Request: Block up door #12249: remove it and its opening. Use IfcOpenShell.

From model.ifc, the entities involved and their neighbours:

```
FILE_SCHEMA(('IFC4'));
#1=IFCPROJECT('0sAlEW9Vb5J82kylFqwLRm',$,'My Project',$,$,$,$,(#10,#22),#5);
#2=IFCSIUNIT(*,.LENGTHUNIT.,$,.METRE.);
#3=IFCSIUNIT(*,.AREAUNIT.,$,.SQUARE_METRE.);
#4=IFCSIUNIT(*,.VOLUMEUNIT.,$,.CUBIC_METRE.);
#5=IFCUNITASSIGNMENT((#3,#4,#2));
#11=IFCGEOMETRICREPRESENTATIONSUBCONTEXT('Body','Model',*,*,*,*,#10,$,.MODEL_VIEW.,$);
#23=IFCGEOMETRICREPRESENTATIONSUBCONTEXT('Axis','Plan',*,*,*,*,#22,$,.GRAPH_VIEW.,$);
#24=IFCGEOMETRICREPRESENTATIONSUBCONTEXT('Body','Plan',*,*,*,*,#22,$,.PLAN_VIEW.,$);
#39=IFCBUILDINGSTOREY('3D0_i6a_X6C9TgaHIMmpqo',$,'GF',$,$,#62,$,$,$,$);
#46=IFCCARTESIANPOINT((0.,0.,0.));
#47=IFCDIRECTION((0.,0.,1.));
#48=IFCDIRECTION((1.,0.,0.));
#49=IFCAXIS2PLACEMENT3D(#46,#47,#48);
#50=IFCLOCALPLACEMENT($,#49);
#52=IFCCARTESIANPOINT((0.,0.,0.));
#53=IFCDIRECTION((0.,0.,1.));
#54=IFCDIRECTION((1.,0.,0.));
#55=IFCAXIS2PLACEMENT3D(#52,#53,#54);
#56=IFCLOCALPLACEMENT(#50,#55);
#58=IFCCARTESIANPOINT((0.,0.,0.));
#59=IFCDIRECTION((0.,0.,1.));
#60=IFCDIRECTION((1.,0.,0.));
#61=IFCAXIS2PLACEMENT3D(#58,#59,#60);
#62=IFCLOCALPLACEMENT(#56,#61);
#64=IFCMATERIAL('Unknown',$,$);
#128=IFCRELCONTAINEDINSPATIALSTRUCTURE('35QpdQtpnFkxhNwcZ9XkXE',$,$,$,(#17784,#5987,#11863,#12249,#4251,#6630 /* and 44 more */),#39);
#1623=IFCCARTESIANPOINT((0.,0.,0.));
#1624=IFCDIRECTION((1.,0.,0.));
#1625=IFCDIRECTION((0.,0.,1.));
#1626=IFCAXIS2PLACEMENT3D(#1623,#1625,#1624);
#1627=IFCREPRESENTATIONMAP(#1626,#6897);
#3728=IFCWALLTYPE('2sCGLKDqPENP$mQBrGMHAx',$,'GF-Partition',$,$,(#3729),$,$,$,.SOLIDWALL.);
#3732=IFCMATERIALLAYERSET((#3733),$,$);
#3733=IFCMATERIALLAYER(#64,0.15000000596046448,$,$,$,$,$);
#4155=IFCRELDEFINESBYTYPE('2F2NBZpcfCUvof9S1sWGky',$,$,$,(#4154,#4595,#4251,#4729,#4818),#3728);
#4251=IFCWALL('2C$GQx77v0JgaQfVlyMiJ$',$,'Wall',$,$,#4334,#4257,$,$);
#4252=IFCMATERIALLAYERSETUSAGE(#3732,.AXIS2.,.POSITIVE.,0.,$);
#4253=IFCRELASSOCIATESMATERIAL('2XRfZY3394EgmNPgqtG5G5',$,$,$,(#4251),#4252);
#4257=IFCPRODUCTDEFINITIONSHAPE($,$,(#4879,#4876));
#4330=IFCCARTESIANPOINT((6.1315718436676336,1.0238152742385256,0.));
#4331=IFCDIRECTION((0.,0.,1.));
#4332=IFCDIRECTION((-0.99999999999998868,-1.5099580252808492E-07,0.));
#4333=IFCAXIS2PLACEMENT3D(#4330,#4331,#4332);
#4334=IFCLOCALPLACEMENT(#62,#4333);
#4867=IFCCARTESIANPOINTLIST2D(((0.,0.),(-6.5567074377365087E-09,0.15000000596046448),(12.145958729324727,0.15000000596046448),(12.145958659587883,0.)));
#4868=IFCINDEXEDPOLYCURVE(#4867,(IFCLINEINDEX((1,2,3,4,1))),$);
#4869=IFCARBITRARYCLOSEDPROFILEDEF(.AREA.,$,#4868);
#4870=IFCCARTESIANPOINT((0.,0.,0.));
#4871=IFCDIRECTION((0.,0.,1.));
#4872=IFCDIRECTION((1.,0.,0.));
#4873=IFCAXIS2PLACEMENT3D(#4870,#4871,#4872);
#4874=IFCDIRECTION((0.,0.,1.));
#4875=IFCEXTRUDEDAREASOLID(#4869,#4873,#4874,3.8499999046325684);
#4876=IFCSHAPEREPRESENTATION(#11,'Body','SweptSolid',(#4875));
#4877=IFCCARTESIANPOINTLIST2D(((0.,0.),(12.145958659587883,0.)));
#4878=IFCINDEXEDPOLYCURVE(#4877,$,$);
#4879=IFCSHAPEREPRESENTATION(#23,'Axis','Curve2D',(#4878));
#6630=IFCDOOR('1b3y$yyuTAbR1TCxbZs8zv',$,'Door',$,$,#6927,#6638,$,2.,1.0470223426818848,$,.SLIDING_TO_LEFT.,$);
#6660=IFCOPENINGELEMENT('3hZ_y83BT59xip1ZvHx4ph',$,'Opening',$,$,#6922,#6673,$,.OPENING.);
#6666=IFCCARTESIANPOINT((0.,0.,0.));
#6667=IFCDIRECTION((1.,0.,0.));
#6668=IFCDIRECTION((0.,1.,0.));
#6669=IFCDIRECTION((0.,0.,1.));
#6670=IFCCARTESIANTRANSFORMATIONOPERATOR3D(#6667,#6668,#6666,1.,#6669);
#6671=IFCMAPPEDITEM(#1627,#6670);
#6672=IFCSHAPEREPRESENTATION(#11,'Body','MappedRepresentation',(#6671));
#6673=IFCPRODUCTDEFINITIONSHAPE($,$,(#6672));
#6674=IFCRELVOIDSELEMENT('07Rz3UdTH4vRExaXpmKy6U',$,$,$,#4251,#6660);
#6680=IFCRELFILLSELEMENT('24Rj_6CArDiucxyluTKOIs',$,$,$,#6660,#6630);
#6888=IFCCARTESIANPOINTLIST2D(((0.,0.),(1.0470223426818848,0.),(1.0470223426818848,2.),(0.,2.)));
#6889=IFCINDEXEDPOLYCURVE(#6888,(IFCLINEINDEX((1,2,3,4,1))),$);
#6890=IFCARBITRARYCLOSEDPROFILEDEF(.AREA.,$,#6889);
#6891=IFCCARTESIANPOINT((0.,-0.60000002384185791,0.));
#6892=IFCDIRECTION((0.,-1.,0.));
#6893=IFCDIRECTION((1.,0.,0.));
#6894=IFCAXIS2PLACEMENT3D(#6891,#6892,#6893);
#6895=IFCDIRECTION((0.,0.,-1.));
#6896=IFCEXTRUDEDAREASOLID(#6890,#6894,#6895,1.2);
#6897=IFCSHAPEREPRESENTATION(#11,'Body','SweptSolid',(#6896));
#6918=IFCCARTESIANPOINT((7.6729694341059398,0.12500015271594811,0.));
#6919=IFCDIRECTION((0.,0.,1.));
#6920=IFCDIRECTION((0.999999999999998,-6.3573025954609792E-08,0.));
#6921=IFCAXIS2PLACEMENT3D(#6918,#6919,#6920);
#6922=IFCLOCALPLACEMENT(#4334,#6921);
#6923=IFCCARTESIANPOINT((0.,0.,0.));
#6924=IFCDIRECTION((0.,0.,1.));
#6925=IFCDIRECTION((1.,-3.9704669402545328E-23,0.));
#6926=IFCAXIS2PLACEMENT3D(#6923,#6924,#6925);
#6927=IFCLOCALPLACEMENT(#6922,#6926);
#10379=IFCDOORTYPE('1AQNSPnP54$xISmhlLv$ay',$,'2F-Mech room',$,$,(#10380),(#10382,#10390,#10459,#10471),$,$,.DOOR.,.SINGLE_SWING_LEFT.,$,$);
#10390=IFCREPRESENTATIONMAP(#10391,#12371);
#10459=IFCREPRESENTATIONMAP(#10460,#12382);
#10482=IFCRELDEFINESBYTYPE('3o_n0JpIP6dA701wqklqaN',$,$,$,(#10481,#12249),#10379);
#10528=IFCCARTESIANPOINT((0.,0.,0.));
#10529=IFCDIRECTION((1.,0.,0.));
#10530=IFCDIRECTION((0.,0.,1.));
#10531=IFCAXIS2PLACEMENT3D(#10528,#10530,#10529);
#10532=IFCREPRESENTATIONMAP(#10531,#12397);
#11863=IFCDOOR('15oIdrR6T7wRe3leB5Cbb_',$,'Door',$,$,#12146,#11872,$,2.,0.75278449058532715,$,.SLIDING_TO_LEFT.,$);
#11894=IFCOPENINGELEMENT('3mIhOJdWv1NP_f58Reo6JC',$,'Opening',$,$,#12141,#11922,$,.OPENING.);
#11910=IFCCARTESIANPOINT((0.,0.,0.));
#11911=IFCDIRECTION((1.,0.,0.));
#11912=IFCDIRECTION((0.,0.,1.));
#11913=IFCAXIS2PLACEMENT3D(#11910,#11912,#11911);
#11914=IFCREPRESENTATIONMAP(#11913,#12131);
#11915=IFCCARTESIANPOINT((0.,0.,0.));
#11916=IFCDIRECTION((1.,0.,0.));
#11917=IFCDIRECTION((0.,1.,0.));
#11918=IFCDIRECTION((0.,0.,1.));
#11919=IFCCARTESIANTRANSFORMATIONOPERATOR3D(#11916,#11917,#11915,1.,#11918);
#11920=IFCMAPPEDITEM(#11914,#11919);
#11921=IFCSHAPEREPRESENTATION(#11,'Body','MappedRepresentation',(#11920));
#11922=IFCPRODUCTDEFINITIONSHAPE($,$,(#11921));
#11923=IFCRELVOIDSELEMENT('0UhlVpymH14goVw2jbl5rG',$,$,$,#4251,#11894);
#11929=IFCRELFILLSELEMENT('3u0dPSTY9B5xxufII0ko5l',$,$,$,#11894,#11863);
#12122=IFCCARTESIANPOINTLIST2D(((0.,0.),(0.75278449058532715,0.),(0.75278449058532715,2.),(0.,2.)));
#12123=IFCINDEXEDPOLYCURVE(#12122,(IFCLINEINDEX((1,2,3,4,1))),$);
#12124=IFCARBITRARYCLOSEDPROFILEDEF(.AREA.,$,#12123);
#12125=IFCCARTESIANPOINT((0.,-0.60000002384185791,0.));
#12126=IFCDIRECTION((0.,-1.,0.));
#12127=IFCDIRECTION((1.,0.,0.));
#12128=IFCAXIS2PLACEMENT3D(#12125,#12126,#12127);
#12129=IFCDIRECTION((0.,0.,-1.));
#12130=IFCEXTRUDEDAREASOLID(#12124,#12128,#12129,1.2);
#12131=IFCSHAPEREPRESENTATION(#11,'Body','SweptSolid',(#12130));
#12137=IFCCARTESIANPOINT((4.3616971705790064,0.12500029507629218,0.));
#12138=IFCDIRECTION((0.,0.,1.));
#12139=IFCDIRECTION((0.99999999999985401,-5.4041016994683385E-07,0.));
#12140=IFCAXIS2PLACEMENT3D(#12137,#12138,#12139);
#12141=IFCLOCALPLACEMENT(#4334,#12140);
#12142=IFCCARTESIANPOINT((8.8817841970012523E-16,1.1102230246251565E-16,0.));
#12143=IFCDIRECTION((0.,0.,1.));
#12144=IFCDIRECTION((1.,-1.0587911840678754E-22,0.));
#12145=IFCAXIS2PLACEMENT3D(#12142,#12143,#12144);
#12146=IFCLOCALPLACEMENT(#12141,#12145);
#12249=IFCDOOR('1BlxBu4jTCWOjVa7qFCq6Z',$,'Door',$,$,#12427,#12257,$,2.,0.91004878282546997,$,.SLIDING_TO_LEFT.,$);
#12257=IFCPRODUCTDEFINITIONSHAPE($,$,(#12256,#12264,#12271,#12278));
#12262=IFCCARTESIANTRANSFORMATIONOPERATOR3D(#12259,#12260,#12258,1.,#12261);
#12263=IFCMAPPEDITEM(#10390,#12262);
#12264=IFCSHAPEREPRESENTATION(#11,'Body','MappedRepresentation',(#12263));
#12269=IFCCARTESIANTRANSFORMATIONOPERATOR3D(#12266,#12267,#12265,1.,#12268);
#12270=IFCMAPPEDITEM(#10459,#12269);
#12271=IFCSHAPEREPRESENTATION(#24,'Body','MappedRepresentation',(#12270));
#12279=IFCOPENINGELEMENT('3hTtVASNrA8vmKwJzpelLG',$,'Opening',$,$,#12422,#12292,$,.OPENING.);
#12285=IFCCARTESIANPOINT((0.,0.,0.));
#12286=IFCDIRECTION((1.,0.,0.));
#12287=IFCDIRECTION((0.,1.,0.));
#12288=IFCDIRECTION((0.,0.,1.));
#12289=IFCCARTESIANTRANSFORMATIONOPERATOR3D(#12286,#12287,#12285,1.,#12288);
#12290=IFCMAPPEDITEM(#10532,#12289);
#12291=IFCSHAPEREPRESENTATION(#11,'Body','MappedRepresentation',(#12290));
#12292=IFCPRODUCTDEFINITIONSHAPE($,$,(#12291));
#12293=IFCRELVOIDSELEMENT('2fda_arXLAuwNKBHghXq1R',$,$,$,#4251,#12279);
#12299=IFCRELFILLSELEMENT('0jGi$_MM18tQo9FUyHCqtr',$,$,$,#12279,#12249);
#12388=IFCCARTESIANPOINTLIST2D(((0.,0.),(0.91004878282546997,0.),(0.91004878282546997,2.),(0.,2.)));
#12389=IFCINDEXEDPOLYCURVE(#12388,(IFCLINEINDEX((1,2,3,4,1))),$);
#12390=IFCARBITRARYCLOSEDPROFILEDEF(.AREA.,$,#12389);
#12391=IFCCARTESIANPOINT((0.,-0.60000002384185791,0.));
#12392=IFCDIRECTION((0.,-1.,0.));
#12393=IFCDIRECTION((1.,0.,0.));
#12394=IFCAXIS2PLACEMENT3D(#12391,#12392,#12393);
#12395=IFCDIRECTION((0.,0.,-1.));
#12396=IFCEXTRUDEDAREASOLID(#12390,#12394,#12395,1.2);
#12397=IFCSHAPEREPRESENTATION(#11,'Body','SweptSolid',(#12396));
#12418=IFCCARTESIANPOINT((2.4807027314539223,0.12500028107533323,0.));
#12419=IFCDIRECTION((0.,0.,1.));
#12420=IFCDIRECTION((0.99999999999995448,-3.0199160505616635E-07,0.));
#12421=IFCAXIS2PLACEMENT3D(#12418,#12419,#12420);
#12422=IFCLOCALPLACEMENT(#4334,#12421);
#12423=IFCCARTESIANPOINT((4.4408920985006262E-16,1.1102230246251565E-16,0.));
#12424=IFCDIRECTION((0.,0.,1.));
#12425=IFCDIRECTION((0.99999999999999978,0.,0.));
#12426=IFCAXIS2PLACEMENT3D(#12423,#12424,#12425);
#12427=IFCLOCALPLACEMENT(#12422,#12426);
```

```python
import ifcopenshell
import ifcopenshell.api.feature
import ifcopenshell.api.root
import ifcopenshell.geom
import ifcopenshell.util.shape

model = ifcopenshell.open("model.ifc")
settings = ifcopenshell.geom.settings()


def volume(element):
    """Net volume in cubic metres, openings subtracted."""
    shape = ifcopenshell.geom.create_shape(settings, element)
    return ifcopenshell.util.shape.get_volume(shape.geometry)


door = model.by_guid("1BlxBu4jTCWOjVa7qFCq6Z")
opening = door.FillsVoids[0].RelatingOpeningElement
wall = opening.VoidsElements[0].RelatingBuildingElement
before = volume(wall)

ifcopenshell.api.root.remove_product(model, product=door)
ifcopenshell.api.feature.remove_feature(model, feature=opening)

after = volume(wall)

print(f"wall volume {before:.3f} -> {after:.3f} m3")

model.write("model_updated.ifc")
```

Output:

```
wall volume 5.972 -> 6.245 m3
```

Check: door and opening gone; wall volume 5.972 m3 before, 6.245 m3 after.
